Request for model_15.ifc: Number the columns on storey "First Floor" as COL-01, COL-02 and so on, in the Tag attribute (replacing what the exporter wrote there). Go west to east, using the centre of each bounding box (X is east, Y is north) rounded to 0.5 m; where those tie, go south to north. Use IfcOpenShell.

First a look at what the model holds.

```python
import ifcopenshell
import ifcopenshell.util.element
import ifcopenshell.util.placement

model = ifcopenshell.open("model_15.ifc")
print(model.schema)
storey = next(s for s in model.by_type("IfcBuildingStorey") if s.Name == "First Floor")
columns = [e for e in ifcopenshell.util.element.get_decomposition(storey) if e.is_a("IfcColumn")]
for e in sorted(columns, key=lambda e: e.id()):
    origin = ifcopenshell.util.placement.get_local_placement(e.ObjectPlacement)[:3, 3]
    print(e.id(), e.Tag, e.Name, origin.round(2) + 0.0, sep=" | ")
```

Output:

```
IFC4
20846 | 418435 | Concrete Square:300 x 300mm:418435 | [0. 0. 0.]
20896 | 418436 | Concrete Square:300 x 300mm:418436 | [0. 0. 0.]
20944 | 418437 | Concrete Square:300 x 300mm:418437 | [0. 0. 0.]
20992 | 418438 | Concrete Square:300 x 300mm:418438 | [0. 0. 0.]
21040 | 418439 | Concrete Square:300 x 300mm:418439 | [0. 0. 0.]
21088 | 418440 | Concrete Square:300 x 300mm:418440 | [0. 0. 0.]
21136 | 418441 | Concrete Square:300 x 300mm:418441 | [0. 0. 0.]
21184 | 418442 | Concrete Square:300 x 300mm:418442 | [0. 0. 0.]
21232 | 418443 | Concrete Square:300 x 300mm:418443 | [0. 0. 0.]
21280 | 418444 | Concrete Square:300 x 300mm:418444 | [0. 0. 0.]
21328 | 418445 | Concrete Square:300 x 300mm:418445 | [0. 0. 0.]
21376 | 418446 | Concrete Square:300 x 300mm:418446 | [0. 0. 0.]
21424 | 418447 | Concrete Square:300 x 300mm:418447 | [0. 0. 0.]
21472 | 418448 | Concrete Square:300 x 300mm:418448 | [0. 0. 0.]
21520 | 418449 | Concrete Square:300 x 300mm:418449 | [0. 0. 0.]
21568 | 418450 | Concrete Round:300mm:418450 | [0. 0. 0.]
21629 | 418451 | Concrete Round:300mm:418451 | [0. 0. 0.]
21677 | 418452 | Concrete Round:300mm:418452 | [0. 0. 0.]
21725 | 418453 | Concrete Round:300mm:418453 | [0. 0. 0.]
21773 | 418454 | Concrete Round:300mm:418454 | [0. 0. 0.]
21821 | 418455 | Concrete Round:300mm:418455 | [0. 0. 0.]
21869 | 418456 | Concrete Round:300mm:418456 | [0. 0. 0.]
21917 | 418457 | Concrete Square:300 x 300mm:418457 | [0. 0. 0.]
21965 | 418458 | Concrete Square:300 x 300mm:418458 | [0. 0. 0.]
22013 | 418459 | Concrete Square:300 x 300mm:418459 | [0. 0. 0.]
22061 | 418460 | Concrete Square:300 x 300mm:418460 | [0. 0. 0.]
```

```python
import ifcopenshell
import ifcopenshell.geom
import ifcopenshell.util.element
import ifcopenshell.util.shape

model = ifcopenshell.open("model_15.ifc")
settings = ifcopenshell.geom.settings()
settings.set("use-world-coords", True)


def centre(element):
    shape = ifcopenshell.geom.create_shape(settings, element)
    return ifcopenshell.util.shape.get_bbox_centroid(shape.geometry)


storey = next(s for s in model.by_type("IfcBuildingStorey") if s.Name == "First Floor")
columns = [e for e in ifcopenshell.util.element.get_decomposition(storey) if e.is_a("IfcColumn")]

# Insertion points can sit at a corner or the storey origin, so sort by the geometry (in metres).
centres = {e: centre(e) for e in columns}
columns.sort(key=lambda e: (round(centres[e][0] / 0.5), centres[e][1]))

for i, e in enumerate(columns, start=1):
    number = f"COL-{i:02d}"
    e.Tag = number
    print(e.id(), number)

model.write("model_15_edited.ifc")
```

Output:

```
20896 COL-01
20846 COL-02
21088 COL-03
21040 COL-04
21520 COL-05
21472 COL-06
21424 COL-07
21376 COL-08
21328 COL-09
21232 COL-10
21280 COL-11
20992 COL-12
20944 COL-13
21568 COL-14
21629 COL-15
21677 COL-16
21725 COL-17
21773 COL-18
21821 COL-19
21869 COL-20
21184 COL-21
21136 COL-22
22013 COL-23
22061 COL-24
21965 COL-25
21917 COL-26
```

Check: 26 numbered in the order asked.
